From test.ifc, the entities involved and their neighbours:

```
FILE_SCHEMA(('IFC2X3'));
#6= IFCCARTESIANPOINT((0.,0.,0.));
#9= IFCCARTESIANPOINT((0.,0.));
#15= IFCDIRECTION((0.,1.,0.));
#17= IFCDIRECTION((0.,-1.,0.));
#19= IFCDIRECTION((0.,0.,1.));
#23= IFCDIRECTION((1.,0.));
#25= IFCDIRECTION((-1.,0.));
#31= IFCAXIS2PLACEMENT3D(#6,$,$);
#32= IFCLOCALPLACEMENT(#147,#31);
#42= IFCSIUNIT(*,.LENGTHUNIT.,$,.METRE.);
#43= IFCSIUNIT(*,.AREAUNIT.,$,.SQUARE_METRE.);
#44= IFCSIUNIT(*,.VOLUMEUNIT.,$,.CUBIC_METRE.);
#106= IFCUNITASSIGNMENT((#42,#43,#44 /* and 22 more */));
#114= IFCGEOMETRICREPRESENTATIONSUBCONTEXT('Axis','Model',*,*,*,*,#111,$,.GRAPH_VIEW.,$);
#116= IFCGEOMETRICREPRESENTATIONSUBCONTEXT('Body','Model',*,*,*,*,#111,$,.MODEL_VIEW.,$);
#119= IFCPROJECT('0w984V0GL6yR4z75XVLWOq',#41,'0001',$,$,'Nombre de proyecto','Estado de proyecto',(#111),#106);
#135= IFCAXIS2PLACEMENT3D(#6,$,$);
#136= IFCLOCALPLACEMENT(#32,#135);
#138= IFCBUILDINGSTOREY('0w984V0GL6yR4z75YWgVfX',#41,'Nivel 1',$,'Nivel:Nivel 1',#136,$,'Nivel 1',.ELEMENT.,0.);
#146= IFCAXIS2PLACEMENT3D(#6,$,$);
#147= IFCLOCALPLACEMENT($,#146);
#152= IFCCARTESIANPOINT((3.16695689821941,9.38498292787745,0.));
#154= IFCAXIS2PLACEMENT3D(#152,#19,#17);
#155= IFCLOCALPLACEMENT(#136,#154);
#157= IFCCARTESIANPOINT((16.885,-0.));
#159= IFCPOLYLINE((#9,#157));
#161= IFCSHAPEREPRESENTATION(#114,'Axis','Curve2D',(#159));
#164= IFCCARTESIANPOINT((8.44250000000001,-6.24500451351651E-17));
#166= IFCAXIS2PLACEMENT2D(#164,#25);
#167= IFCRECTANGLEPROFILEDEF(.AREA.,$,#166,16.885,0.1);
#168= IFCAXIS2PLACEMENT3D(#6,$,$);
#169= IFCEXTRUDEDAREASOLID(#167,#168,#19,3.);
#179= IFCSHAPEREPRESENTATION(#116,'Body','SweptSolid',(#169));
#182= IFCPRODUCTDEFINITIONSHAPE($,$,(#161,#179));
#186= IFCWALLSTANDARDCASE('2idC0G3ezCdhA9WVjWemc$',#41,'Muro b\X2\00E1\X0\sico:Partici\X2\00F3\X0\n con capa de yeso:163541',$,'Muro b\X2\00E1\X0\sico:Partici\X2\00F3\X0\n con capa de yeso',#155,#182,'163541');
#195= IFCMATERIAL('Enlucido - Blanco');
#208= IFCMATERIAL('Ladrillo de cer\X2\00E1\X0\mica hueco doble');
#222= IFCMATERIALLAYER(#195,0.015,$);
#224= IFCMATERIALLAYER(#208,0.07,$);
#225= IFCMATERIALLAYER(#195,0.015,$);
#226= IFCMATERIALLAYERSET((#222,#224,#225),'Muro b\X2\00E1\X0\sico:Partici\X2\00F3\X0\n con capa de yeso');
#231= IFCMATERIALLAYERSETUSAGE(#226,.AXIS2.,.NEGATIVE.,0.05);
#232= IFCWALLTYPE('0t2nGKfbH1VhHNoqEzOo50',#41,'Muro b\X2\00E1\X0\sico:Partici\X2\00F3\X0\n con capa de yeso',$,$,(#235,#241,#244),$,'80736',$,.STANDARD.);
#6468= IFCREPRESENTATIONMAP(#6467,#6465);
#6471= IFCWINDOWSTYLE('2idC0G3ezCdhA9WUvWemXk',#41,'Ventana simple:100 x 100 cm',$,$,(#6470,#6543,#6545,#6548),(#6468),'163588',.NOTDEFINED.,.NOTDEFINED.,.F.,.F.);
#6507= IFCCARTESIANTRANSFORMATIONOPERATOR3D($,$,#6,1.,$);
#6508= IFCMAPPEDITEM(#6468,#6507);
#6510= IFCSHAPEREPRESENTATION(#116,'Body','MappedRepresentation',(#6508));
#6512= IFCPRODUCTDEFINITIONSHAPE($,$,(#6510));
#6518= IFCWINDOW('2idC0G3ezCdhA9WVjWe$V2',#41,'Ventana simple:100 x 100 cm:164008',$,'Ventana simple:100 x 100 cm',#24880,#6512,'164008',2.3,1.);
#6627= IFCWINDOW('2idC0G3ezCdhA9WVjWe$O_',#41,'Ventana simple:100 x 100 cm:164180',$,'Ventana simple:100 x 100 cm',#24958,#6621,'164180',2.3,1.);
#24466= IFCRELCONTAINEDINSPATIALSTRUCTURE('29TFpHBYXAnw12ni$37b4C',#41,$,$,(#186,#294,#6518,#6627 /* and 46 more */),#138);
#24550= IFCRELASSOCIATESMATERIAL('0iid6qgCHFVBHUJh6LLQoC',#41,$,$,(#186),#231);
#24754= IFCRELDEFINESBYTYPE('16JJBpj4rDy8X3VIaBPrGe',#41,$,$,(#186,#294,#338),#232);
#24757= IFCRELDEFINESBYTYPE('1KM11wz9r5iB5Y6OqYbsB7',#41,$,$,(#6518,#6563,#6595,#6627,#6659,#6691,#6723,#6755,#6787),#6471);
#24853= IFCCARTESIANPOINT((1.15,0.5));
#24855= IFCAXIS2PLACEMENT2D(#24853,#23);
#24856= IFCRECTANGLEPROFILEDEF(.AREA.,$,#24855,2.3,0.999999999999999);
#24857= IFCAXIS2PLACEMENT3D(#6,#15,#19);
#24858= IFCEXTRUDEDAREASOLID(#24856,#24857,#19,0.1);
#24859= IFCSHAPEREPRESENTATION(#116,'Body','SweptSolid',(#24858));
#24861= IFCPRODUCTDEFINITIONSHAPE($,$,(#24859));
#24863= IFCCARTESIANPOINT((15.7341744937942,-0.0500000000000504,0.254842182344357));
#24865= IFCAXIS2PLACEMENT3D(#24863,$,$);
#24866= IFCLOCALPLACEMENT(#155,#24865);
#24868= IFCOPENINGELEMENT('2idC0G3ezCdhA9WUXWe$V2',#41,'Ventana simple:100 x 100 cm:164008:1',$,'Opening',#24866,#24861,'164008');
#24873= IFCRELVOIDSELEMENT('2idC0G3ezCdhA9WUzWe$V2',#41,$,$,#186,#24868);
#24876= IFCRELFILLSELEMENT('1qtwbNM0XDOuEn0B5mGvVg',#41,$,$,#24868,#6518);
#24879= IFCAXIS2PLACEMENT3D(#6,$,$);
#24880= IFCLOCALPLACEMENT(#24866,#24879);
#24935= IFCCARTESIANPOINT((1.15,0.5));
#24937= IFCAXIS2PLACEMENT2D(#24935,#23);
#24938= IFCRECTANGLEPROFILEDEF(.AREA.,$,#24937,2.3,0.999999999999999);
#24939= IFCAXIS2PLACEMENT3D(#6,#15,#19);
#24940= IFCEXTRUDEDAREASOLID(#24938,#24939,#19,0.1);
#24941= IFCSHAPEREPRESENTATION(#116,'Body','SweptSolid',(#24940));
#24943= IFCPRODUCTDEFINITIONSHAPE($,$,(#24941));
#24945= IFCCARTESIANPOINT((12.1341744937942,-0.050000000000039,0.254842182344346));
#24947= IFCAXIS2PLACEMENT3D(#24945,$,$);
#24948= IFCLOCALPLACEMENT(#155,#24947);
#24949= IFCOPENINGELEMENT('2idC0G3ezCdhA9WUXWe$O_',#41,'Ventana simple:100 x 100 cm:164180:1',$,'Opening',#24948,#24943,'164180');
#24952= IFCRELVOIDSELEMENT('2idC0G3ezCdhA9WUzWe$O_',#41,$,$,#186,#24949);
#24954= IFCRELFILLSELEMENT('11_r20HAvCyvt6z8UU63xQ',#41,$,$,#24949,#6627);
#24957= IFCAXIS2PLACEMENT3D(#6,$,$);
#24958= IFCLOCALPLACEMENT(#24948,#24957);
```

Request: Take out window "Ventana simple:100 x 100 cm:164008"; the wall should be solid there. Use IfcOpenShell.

```python
import ifcopenshell
import ifcopenshell.api.feature
import ifcopenshell.api.root
import ifcopenshell.geom
import ifcopenshell.util.shape

model = ifcopenshell.open("test.ifc")
settings = ifcopenshell.geom.settings()


def volume(element):
    """Net volume in cubic metres, openings subtracted."""
    shape = ifcopenshell.geom.create_shape(settings, element)
    return ifcopenshell.util.shape.get_volume(shape.geometry)


window = model.by_id(6518)
opening = window.FillsVoids[0].RelatingOpeningElement
wall = opening.VoidsElements[0].RelatingBuildingElement
before = volume(wall)

ifcopenshell.api.root.remove_product(model, product=window)
ifcopenshell.api.feature.remove_feature(model, feature=opening)

after = volume(wall)

print(f"wall volume {before:.3f} -> {after:.3f} m3")

model.write("test_edited.ifc")
```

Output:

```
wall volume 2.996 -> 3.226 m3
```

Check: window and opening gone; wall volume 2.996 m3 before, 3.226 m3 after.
